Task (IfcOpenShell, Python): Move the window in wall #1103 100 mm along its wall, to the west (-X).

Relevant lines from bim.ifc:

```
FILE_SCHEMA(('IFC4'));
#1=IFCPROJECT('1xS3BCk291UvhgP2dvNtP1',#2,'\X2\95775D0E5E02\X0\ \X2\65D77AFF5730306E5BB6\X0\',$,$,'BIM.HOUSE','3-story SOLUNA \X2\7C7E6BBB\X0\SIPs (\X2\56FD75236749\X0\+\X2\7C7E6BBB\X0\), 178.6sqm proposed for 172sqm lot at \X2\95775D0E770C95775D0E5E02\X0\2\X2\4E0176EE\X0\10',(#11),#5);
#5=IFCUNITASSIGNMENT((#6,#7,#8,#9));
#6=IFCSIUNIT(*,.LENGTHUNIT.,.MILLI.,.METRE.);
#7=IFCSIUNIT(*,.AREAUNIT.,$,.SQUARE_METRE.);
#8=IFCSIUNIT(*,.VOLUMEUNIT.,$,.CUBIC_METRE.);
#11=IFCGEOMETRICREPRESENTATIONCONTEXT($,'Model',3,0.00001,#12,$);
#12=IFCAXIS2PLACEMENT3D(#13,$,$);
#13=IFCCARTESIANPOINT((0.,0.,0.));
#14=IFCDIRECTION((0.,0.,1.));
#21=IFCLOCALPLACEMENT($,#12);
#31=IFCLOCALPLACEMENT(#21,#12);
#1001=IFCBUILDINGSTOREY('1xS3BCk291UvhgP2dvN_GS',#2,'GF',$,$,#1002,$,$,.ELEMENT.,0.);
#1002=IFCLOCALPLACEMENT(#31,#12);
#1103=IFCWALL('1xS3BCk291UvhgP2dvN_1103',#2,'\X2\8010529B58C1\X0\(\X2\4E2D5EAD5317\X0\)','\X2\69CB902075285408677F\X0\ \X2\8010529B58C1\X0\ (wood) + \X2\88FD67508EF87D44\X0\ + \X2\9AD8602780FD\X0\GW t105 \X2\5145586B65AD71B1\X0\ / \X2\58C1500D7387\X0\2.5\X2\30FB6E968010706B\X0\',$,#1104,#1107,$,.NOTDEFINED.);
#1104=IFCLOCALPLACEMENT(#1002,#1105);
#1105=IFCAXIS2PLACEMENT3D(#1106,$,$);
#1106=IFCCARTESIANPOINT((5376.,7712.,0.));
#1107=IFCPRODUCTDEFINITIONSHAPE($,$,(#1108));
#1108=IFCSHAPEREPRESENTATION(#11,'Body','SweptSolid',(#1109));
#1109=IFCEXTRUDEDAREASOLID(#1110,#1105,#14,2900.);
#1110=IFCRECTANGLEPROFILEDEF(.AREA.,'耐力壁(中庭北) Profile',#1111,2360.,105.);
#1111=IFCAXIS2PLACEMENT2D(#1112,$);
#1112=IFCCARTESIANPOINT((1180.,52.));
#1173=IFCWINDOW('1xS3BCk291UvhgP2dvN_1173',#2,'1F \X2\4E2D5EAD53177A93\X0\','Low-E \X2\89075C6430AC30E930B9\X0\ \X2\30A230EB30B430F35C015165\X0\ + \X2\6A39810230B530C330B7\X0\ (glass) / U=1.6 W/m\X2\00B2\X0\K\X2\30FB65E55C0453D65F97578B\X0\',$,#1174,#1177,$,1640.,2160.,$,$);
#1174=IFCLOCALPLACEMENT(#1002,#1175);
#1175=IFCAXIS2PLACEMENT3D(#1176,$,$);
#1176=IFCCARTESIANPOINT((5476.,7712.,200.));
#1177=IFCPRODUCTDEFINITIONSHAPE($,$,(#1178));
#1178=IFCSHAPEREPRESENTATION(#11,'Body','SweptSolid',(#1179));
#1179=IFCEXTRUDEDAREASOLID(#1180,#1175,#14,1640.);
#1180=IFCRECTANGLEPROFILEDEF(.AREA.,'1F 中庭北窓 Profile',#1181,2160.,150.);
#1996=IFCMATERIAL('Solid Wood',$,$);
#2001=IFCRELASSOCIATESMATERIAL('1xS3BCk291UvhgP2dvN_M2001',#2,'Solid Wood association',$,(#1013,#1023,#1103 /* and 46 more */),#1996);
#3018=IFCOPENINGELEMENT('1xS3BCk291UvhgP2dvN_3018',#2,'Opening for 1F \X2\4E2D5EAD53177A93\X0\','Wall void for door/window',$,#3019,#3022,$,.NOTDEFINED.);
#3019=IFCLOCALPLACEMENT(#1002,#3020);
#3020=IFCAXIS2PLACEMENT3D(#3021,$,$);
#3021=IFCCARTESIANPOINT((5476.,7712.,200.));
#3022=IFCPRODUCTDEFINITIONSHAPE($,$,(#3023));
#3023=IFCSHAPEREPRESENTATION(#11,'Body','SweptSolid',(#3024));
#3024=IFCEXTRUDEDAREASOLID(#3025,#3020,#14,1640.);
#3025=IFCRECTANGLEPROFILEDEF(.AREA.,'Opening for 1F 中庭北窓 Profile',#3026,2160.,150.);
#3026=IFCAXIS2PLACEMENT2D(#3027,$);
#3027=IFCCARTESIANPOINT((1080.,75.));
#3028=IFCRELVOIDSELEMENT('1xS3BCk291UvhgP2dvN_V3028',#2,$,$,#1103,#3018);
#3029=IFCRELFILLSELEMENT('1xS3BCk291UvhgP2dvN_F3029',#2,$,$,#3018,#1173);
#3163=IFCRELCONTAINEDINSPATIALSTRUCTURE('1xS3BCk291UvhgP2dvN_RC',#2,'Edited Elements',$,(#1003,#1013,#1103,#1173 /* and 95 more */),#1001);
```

```python
import ifcopenshell
import ifcopenshell.api.geometry
import ifcopenshell.util.placement

model = ifcopenshell.open("bim.ifc")

window = model.by_id(1173)
opening = window.FillsVoids[0].RelatingOpeningElement
wall = opening.VoidsElements[0].RelatingBuildingElement

wall_matrix = ifcopenshell.util.placement.get_local_placement(wall.ObjectPlacement)
shift = wall_matrix[:3, 0] * -100.0
before = ifcopenshell.util.placement.get_local_placement(window.ObjectPlacement)[:3, 3].copy()

# The window is not placed relative to its opening, so move both.
for product in (opening, window):
    matrix = ifcopenshell.util.placement.get_local_placement(product.ObjectPlacement)
    matrix[:3, 3] += shift
    ifcopenshell.api.geometry.edit_object_placement(model, product=product, matrix=matrix, is_si=False)

after = ifcopenshell.util.placement.get_local_placement(window.ObjectPlacement)[:3, 3]
print("window moved by", (after - before).round(3) + 0.0)

model.write("bim-out.ifc")
```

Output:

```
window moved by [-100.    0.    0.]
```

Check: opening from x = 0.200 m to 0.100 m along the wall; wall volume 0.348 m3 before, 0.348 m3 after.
